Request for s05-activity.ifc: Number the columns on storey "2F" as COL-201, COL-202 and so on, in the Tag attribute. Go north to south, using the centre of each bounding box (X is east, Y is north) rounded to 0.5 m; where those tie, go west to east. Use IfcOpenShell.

First a look at what the model holds.

```python
import ifcopenshell
import ifcopenshell.util.element
import ifcopenshell.util.placement

model = ifcopenshell.open("s05-activity.ifc")
print(model.schema)
storey = next(s for s in model.by_type("IfcBuildingStorey") if s.Name == "2F")
columns = [e for e in ifcopenshell.util.element.get_decomposition(storey) if e.is_a("IfcColumn")]
for e in sorted(columns, key=lambda e: e.id()):
    origin = ifcopenshell.util.placement.get_local_placement(e.ObjectPlacement)[:3, 3]
    print(e.id(), e.Tag, e.Name, origin.round(2) + 0.0, sep=" | ")
```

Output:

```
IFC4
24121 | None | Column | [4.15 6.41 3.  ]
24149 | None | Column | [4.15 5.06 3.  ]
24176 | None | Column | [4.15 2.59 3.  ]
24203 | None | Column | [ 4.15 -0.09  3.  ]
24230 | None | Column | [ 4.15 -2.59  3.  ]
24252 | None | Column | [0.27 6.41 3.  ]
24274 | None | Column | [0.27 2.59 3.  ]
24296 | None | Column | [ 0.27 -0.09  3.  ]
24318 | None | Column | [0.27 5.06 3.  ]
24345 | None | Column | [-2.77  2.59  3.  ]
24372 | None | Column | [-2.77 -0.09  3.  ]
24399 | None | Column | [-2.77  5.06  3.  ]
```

```python
import ifcopenshell
import ifcopenshell.geom
import ifcopenshell.util.element
import ifcopenshell.util.shape

model = ifcopenshell.open("s05-activity.ifc")
settings = ifcopenshell.geom.settings()
settings.set("use-world-coords", True)


def centre(element):
    shape = ifcopenshell.geom.create_shape(settings, element)
    return ifcopenshell.util.shape.get_bbox_centroid(shape.geometry)


storey = next(s for s in model.by_type("IfcBuildingStorey") if s.Name == "2F")
columns = [e for e in ifcopenshell.util.element.get_decomposition(storey) if e.is_a("IfcColumn")]

# Insertion points can sit at a corner or the storey origin, so sort by the geometry (in metres).
centres = {e: centre(e) for e in columns}
columns.sort(key=lambda e: (-round(centres[e][1] / 0.5), centres[e][0]))

for i, e in enumerate(columns, start=1):
    number = f"COL-2{i:02d}"
    e.Tag = number
    print(e.id(), number)

model.write("s05-activity_edited.ifc")
```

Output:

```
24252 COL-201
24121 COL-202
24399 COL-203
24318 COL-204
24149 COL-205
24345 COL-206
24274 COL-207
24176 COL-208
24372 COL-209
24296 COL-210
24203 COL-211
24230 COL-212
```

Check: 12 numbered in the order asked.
